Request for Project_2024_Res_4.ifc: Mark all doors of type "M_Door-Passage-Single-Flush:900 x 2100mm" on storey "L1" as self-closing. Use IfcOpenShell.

First a look at what the model holds.

```python
import ifcopenshell
import ifcopenshell.util.element

model = ifcopenshell.open("Project_2024_Res_4.ifc")
print(model.schema)
storey = next(s for s in model.by_type("IfcBuildingStorey") if s.Name == "L1")
doors = [e for e in ifcopenshell.util.element.get_decomposition(storey) if e.is_a("IfcDoor")]
seen = {}
for e in doors:
    element_type = ifcopenshell.util.element.get_type(e)
    key = (element_type.Name if element_type != e and element_type else None, ifcopenshell.util.element.get_pset(e, "Pset_DoorCommon", "SelfClosing"))
    seen[key] = seen.get(key, 0) + 1
for (name, value), count in sorted(seen.items(), key=str):
    print(count, "x", name, "|", value)
```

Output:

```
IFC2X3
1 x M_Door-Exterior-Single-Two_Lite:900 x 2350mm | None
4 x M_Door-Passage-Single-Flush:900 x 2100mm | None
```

```python
import ifcopenshell
import ifcopenshell.api.pset
import ifcopenshell.util.element

model = ifcopenshell.open("Project_2024_Res_4.ifc")

storey = next(s for s in model.by_type("IfcBuildingStorey") if s.Name == "L1")
doors = [e for e in ifcopenshell.util.element.get_decomposition(storey) if e.is_a("IfcDoor")]

count = 0
for e in doors:
    element_type = ifcopenshell.util.element.get_type(e)
    if element_type in (None, e) or element_type.Name != "M_Door-Passage-Single-Flush:900 x 2100mm":
        continue
    # add_pset returns the element's existing set when there is one.
    pset = ifcopenshell.api.pset.add_pset(model, product=e, name="Pset_DoorCommon")
    ifcopenshell.api.pset.edit_pset(model, pset=pset, properties={"SelfClosing": True})
    count += 1

print(count, "doors updated")

model.write("Project_2024_Res_4_edited.ifc")
```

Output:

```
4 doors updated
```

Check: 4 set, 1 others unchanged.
